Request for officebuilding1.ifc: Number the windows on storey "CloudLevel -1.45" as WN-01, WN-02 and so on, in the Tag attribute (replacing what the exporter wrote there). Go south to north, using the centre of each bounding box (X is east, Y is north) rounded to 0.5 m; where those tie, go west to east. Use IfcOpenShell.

First a look at what the model holds.

```python
import ifcopenshell
import ifcopenshell.util.element
import ifcopenshell.util.placement

model = ifcopenshell.open("officebuilding1.ifc")
print(model.schema)
storey = next(s for s in model.by_type("IfcBuildingStorey") if s.Name == "CloudLevel -1.45")
windows = [e for e in ifcopenshell.util.element.get_decomposition(storey) if e.is_a("IfcWindow")]
for e in sorted(windows, key=lambda e: e.id()):
    origin = ifcopenshell.util.placement.get_local_placement(e.ObjectPlacement)[:3, 3]
    print(e.id(), e.Tag, e.Name, origin.round(2) + 0.0, sep=" | ")
```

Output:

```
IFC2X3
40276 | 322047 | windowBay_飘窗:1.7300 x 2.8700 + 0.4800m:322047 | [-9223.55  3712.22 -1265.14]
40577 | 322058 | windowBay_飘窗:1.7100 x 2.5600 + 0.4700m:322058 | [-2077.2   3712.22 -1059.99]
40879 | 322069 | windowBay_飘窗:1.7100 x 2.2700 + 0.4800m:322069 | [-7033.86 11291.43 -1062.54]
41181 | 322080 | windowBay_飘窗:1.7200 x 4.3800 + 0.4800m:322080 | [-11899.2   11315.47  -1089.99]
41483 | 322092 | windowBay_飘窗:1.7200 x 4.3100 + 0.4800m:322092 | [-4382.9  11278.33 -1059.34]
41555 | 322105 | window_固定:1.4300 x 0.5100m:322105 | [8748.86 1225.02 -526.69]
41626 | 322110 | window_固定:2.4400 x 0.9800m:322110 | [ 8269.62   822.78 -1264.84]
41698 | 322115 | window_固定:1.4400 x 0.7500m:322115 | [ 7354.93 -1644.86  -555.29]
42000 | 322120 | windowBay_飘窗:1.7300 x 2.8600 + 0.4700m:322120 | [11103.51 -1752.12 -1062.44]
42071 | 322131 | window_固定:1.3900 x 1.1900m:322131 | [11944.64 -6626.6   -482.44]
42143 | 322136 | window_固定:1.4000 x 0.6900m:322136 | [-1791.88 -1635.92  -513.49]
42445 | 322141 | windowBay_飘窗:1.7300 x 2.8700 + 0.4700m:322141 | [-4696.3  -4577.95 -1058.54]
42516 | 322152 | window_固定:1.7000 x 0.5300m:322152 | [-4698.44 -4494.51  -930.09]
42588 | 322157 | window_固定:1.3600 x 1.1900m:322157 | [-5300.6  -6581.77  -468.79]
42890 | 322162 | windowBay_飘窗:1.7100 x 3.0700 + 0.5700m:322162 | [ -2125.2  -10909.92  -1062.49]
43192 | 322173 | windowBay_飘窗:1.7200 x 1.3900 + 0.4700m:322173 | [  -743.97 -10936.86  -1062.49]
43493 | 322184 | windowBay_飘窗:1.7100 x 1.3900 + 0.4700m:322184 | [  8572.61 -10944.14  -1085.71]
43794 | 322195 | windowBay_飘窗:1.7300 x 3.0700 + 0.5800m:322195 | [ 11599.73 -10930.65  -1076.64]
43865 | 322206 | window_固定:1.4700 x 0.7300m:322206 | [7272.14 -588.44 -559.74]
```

```python
import ifcopenshell
import ifcopenshell.geom
import ifcopenshell.util.element
import ifcopenshell.util.shape

model = ifcopenshell.open("officebuilding1.ifc")
settings = ifcopenshell.geom.settings()
settings.set("use-world-coords", True)


def centre(element):
    shape = ifcopenshell.geom.create_shape(settings, element)
    return ifcopenshell.util.shape.get_bbox_centroid(shape.geometry)


storey = next(s for s in model.by_type("IfcBuildingStorey") if s.Name == "CloudLevel -1.45")
windows = [e for e in ifcopenshell.util.element.get_decomposition(storey) if e.is_a("IfcWindow")]

# Insertion points can sit at a corner or the storey origin, so sort by the geometry (in metres).
centres = {e: centre(e) for e in windows}
windows.sort(key=lambda e: (round(centres[e][1] / 0.5), centres[e][0]))

for i, e in enumerate(windows, start=1):
    number = f"WN-{i:02d}"
    e.Tag = number
    print(e.id(), number)

model.write("officebuilding1_rev.ifc")
```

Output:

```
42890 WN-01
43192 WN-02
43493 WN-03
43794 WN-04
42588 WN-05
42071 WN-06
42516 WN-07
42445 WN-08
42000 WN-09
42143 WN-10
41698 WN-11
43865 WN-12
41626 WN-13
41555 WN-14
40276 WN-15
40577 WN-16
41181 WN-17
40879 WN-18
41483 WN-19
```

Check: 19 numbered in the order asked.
